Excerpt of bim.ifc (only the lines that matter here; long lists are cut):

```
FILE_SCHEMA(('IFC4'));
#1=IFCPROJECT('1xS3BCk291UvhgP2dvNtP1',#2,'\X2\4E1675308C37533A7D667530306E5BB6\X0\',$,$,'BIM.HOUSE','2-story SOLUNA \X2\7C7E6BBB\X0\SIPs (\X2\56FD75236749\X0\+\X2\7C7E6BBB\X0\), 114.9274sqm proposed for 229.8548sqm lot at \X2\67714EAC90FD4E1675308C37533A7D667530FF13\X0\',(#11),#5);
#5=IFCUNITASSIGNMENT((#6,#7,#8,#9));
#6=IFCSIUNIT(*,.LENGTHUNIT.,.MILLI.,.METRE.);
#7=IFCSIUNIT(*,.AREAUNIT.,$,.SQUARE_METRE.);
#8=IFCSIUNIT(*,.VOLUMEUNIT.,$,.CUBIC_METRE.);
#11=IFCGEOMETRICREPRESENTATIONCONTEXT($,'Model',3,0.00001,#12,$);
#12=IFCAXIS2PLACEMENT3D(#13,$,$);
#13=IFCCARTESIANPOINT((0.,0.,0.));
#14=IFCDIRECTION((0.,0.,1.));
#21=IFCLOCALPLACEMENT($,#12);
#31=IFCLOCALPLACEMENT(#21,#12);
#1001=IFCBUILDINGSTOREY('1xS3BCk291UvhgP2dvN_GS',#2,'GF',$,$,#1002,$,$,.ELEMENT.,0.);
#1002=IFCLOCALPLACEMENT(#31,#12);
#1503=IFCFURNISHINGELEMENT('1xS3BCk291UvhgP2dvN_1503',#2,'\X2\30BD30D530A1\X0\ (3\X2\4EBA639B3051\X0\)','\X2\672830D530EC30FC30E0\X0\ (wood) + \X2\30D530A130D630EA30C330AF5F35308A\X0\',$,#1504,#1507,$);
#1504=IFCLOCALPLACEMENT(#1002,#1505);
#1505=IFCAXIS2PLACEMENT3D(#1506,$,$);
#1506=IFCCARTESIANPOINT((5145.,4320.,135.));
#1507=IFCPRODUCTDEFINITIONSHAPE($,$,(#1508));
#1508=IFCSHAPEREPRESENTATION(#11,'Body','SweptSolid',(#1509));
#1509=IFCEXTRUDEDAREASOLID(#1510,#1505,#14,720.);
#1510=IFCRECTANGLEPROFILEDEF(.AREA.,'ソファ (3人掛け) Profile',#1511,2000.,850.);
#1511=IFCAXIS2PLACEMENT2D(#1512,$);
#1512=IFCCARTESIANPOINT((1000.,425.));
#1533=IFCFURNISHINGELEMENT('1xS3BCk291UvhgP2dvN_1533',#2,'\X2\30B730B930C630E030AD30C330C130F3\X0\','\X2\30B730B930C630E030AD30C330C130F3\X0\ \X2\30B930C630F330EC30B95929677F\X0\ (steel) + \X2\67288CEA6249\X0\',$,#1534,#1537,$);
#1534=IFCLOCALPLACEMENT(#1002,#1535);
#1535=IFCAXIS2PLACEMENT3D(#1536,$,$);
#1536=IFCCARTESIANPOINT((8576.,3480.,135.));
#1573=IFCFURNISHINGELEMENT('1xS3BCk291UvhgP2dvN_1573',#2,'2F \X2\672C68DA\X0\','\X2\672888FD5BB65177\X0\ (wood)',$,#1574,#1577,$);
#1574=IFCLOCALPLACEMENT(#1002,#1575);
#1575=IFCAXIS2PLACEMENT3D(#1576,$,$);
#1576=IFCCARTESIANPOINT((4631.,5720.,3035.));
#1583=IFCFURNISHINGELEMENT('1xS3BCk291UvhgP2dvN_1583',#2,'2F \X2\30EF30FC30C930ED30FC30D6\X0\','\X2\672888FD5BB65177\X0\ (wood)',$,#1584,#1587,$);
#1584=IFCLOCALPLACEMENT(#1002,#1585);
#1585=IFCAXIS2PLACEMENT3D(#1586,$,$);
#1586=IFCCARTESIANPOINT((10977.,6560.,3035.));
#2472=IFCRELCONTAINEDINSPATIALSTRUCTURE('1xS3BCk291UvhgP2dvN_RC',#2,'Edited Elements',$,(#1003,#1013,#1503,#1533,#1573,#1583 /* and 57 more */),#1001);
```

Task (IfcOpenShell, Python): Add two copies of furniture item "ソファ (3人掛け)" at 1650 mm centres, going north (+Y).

```python
import numpy as np
import ifcopenshell
import ifcopenshell.api.geometry
import ifcopenshell.api.root
import ifcopenshell.util.element
import ifcopenshell.util.placement
import ifcopenshell.util.unit

model = ifcopenshell.open("bim.ifc")
unit_scale = ifcopenshell.util.unit.calculate_unit_scale(model)


def reuse_history(source, copy):
    """copy_class also copies each property set's owner history, people and application; keep the originals."""
    for rel in copy.IsDefinedBy:
        if rel.is_a("IfcRelDefinesByProperties") and (history := rel.RelatingPropertyDefinition.OwnerHistory):
            rel.RelatingPropertyDefinition.OwnerHistory = source.OwnerHistory
            ifcopenshell.util.element.remove_deep2(model, history)


source = model.by_guid("1xS3BCk291UvhgP2dvN_1503")
base = ifcopenshell.util.placement.get_local_placement(source.ObjectPlacement)
step = np.array([0.0, 1.0, 0.0]) * 1.65 / unit_scale

for i in range(1, 3):
    copy = ifcopenshell.api.root.copy_class(model, product=source)
    copy.Representation = ifcopenshell.util.element.copy_deep(
        model, source.Representation, exclude=["IfcGeometricRepresentationContext", "IfcRepresentationMap"]
    )
    reuse_history(source, copy)
    matrix = base.copy()
    matrix[:3, 3] += i * step
    print("added at", matrix[:3, 3].round(3) + 0.0)
    ifcopenshell.api.geometry.edit_object_placement(model, product=copy, matrix=matrix, is_si=False)

model.write("bim_v2.ifc")
```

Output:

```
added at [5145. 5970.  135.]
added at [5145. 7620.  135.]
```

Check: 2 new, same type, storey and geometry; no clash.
